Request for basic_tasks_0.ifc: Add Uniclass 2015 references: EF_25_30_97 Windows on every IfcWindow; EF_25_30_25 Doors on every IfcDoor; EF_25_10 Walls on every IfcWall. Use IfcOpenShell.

First a look at what the model holds.

```python
import ifcopenshell

model = ifcopenshell.open("basic_tasks_0.ifc")
print(model.schema)
print("classifications:", [c.Name for c in model.by_type("IfcClassification")])
for ifc_class in ("IfcDoor", "IfcRoof", "IfcStair", "IfcWall", "IfcWindow"):
    print(ifc_class, len(model.by_type(ifc_class)))
```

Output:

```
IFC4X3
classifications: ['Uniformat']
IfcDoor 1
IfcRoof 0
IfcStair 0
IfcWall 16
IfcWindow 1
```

```python
import ifcopenshell
import ifcopenshell.api.classification

model = ifcopenshell.open("basic_tasks_0.ifc")

system = ifcopenshell.api.classification.add_classification(model, classification="Uniclass 2015")

codes = {
    "IfcWindow": ("EF_25_30_97", "Windows"),
    "IfcDoor": ("EF_25_30_25", "Doors"),
    "IfcWall": ("EF_25_10", "Walls"),
}
for ifc_class, (code, name) in codes.items():
    products = model.by_type(ifc_class)
    ifcopenshell.api.classification.add_reference(
        model, products=products, classification=system, identification=code, name=name
    )
    print(code, len(products))

model.write("basic_tasks_0_rev.ifc")
```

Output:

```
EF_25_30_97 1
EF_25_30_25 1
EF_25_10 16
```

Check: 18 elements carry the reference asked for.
